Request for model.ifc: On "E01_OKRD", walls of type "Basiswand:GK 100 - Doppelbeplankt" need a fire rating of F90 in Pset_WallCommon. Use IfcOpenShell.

First a look at what the model holds.

```python
import ifcopenshell
import ifcopenshell.util.element

model = ifcopenshell.open("model.ifc")
print(model.schema)
storey = next(s for s in model.by_type("IfcBuildingStorey") if s.Name == "E01_OKRD")
walls = [e for e in ifcopenshell.util.element.get_decomposition(storey) if e.is_a("IfcWall")]
seen = {}
for e in walls:
    element_type = ifcopenshell.util.element.get_type(e)
    key = (element_type.Name if element_type != e and element_type else None, ifcopenshell.util.element.get_pset(e, "Pset_WallCommon", "FireRating"))
    seen[key] = seen.get(key, 0) + 1
for (name, value), count in sorted(seen.items(), key=str):
    print(count, "x", name, "|", value)
```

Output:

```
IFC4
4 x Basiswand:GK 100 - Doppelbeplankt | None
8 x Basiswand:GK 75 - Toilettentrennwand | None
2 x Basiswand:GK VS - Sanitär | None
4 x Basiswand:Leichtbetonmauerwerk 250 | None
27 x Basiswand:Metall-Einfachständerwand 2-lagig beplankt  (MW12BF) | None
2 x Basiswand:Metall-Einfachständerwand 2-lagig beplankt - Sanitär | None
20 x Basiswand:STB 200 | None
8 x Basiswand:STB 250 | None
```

```python
import ifcopenshell
import ifcopenshell.api.pset
import ifcopenshell.util.element

model = ifcopenshell.open("model.ifc")

storey = next(s for s in model.by_type("IfcBuildingStorey") if s.Name == "E01_OKRD")
walls = [e for e in ifcopenshell.util.element.get_decomposition(storey) if e.is_a("IfcWall")]

count = 0
for e in walls:
    element_type = ifcopenshell.util.element.get_type(e)
    if element_type in (None, e) or element_type.Name != "Basiswand:GK 100 - Doppelbeplankt":
        continue
    # add_pset returns the element's existing set when there is one.
    pset = ifcopenshell.api.pset.add_pset(model, product=e, name="Pset_WallCommon")
    ifcopenshell.api.pset.edit_pset(model, pset=pset, properties={"FireRating": "F90"})
    count += 1

print(count, "walls updated")

model.write("model_updated.ifc")
```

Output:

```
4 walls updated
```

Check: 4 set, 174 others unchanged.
